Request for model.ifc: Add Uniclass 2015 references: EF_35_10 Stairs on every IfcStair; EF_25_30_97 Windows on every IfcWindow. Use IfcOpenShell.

First a look at what the model holds.

```python
import ifcopenshell

model = ifcopenshell.open("model.ifc")
print(model.schema)
print("classifications:", [c.Name for c in model.by_type("IfcClassification")])
for ifc_class in ("IfcDoor", "IfcRoof", "IfcStair", "IfcWall", "IfcWindow"):
    print(ifc_class, len(model.by_type(ifc_class)))
```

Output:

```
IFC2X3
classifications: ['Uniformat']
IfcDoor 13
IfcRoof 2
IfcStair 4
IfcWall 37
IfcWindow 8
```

```python
import ifcopenshell
import ifcopenshell.api.classification

model = ifcopenshell.open("model.ifc")

# IFC2X3 requires Source and Edition and has no link from the project to the system.
system = model.create_entity("IfcClassification", Source="NBS", Edition="2015", Name="Uniclass 2015")

codes = {
    "IfcStair": ("EF_35_10", "Stairs"),
    "IfcWindow": ("EF_25_30_97", "Windows"),
}
for ifc_class, (code, name) in codes.items():
    products = model.by_type(ifc_class)
    ifcopenshell.api.classification.add_reference(
        model, products=products, classification=system, identification=code, name=name
    )
    print(code, len(products))

model.write("model-out.ifc")
```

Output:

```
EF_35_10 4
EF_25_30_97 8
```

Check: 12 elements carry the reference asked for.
